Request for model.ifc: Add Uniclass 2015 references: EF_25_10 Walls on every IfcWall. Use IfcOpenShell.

First a look at what the model holds.

```python
import ifcopenshell

model = ifcopenshell.open("model.ifc")
print(model.schema)
print("classifications:", [c.Name for c in model.by_type("IfcClassification")])
for ifc_class in ("IfcDoor", "IfcRoof", "IfcStair", "IfcWall", "IfcWindow"):
    print(ifc_class, len(model.by_type(ifc_class)))
```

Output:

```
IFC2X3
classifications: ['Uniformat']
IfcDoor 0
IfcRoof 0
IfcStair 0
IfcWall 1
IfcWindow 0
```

```python
import ifcopenshell
import ifcopenshell.api.classification

model = ifcopenshell.open("model.ifc")

# IFC2X3 requires Source and Edition and has no link from the project to the system.
system = model.create_entity("IfcClassification", Source="NBS", Edition="2015", Name="Uniclass 2015")

codes = {
    "IfcWall": ("EF_25_10", "Walls"),
}
for ifc_class, (code, name) in codes.items():
    products = model.by_type(ifc_class)
    ifcopenshell.api.classification.add_reference(
        model, products=products, classification=system, identification=code, name=name
    )
    print(code, len(products))

model.write("model_updated.ifc")
```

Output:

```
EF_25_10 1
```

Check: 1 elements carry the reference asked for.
